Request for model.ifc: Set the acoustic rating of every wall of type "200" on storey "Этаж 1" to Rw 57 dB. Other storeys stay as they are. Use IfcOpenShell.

First a look at what the model holds.

```python
import ifcopenshell
import ifcopenshell.util.element

model = ifcopenshell.open("model.ifc")
print(model.schema)
storey = next(s for s in model.by_type("IfcBuildingStorey") if s.Name == "Этаж 1")
walls = [e for e in ifcopenshell.util.element.get_decomposition(storey) if e.is_a("IfcWall")]
seen = {}
for e in walls:
    element_type = ifcopenshell.util.element.get_type(e)
    key = (element_type.Name if element_type != e and element_type else None, ifcopenshell.util.element.get_pset(e, "Pset_WallCommon", "AcousticRating"))
    seen[key] = seen.get(key, 0) + 1
for (name, value), count in sorted(seen.items(), key=str):
    print(count, "x", name, "|", value)
```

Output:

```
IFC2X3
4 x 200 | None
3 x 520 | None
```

```python
import ifcopenshell
import ifcopenshell.api.pset
import ifcopenshell.util.element

model = ifcopenshell.open("model.ifc")

storey = next(s for s in model.by_type("IfcBuildingStorey") if s.Name == "Этаж 1")
walls = [e for e in ifcopenshell.util.element.get_decomposition(storey) if e.is_a("IfcWall")]

count = 0
for e in walls:
    element_type = ifcopenshell.util.element.get_type(e)
    if element_type in (None, e) or element_type.Name != "200":
        continue
    # add_pset returns the element's existing set when there is one.
    pset = ifcopenshell.api.pset.add_pset(model, product=e, name="Pset_WallCommon")
    ifcopenshell.api.pset.edit_pset(model, pset=pset, properties={"AcousticRating": "Rw 57 dB"})
    count += 1

print(count, "walls updated")

model.write("model-out.ifc")
```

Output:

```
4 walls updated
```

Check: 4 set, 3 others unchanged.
